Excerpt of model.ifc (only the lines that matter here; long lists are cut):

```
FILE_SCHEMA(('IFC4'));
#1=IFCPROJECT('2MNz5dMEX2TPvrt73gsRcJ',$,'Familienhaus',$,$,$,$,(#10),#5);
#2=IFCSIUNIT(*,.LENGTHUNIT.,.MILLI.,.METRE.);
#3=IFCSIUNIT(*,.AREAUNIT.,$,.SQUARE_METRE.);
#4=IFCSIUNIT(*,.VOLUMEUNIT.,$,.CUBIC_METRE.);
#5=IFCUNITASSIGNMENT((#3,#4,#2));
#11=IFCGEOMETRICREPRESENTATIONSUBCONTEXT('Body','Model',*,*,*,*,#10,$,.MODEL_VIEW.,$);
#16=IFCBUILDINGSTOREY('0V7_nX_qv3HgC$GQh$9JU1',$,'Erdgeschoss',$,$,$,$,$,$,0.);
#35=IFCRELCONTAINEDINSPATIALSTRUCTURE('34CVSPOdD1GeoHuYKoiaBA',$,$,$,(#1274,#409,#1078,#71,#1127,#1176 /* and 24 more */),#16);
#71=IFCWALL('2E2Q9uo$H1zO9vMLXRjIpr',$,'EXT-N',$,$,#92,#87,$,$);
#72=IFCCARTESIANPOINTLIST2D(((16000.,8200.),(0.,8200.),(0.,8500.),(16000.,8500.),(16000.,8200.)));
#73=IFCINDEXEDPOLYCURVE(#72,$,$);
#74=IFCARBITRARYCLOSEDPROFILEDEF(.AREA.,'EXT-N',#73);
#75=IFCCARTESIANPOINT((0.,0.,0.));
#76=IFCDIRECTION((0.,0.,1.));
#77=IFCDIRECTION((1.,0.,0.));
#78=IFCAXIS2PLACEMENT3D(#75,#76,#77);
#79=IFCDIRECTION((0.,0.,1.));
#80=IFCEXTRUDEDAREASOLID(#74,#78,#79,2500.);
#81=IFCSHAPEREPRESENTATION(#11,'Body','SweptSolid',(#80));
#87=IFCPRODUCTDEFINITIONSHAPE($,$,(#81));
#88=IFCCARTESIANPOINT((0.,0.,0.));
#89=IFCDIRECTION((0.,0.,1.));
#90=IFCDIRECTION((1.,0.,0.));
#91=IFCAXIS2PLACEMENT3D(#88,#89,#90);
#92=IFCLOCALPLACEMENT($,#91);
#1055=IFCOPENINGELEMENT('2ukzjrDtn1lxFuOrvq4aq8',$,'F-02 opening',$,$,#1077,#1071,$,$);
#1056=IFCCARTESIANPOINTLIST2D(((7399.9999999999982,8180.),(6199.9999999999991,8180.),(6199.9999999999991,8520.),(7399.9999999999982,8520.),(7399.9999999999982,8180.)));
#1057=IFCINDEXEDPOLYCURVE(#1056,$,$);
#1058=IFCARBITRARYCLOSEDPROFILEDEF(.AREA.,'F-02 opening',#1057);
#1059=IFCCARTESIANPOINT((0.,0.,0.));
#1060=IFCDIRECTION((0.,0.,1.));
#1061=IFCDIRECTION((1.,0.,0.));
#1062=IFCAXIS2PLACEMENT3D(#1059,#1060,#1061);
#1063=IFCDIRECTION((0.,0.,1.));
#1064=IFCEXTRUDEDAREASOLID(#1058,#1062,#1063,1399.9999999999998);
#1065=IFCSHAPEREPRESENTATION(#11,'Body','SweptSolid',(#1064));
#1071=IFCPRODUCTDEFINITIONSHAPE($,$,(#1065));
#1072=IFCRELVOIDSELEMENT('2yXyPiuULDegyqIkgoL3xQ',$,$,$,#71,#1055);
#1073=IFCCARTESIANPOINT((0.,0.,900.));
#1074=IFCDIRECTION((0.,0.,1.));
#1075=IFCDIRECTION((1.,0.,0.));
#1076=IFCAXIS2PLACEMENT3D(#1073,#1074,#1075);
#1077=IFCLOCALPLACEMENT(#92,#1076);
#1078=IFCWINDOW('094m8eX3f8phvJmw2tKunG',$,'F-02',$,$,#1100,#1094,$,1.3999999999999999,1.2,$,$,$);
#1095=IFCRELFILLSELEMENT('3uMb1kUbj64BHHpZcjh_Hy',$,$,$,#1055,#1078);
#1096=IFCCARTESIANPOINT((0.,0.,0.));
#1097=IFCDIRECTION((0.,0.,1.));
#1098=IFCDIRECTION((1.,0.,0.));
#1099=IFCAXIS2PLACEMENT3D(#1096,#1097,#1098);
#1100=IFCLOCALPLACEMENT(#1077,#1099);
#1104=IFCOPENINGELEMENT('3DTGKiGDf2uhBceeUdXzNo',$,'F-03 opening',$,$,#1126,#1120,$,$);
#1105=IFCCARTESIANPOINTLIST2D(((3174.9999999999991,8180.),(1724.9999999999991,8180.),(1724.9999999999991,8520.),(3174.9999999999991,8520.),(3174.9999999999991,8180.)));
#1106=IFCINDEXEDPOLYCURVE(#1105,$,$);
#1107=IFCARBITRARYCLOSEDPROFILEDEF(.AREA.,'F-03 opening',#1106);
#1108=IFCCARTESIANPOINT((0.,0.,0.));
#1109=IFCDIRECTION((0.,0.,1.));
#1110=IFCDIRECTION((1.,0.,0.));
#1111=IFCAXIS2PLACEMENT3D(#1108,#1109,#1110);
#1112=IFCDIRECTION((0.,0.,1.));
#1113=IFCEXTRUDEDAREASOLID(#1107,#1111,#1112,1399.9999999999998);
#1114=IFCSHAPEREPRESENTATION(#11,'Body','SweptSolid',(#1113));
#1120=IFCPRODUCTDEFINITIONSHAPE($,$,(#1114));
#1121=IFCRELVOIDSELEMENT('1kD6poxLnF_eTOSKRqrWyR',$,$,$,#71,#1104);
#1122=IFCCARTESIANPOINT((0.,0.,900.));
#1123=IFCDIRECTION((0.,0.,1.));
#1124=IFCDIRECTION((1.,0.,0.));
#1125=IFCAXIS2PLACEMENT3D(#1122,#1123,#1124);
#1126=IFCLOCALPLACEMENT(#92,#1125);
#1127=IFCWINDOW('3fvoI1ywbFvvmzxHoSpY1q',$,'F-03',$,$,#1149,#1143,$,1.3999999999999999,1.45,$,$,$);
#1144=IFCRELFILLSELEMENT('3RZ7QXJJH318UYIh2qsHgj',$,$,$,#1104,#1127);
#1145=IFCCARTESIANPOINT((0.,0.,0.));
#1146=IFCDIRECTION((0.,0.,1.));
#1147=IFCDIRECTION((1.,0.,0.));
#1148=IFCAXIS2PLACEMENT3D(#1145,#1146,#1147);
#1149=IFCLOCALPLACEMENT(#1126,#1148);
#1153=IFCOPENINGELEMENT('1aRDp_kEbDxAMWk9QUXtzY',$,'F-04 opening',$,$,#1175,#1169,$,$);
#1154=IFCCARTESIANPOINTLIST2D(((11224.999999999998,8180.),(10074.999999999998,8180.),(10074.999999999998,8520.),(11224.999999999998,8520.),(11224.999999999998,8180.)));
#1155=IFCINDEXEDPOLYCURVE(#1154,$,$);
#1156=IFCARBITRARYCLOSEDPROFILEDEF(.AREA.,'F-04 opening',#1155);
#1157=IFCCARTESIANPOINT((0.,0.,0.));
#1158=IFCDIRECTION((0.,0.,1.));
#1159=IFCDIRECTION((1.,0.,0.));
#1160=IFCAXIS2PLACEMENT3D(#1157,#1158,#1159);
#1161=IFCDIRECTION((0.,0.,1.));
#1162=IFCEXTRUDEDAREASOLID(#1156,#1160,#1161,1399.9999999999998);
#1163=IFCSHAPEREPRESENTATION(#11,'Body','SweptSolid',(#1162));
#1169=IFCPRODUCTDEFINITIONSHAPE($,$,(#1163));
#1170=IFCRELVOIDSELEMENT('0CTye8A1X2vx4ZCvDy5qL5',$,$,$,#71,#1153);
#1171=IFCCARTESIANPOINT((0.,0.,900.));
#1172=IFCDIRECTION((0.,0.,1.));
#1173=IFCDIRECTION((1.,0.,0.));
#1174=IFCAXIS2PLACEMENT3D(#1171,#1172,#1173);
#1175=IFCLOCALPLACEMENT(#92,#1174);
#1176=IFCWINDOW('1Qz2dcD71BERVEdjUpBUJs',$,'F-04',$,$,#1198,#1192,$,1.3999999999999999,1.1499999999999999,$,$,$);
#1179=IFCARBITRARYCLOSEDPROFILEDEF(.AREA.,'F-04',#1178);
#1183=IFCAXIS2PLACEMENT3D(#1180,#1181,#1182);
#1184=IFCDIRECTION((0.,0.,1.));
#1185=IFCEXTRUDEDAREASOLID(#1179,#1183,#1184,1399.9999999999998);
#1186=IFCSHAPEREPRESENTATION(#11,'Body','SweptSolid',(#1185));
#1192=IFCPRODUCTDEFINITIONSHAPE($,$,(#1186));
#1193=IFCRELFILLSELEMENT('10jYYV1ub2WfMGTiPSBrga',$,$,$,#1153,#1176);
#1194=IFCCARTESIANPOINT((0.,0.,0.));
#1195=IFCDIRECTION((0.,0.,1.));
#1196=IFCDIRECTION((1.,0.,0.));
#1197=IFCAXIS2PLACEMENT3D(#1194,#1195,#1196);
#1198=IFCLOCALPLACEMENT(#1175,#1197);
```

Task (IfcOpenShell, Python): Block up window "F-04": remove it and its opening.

```python
import ifcopenshell
import ifcopenshell.api.feature
import ifcopenshell.api.root
import ifcopenshell.geom
import ifcopenshell.util.shape

model = ifcopenshell.open("model.ifc")
settings = ifcopenshell.geom.settings()


def volume(element):
    """Net volume in cubic metres, openings subtracted."""
    shape = ifcopenshell.geom.create_shape(settings, element)
    return ifcopenshell.util.shape.get_volume(shape.geometry)


window = model.by_guid("1Qz2dcD71BERVEdjUpBUJs")
opening = window.FillsVoids[0].RelatingOpeningElement
wall = opening.VoidsElements[0].RelatingBuildingElement
before = volume(wall)

ifcopenshell.api.root.remove_product(model, product=window)
ifcopenshell.api.feature.remove_feature(model, feature=opening)

after = volume(wall)

print(f"wall volume {before:.3f} -> {after:.3f} m3")

model.write("model_v2.ifc")
```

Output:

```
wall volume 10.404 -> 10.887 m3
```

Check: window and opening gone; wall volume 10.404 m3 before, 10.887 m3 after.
